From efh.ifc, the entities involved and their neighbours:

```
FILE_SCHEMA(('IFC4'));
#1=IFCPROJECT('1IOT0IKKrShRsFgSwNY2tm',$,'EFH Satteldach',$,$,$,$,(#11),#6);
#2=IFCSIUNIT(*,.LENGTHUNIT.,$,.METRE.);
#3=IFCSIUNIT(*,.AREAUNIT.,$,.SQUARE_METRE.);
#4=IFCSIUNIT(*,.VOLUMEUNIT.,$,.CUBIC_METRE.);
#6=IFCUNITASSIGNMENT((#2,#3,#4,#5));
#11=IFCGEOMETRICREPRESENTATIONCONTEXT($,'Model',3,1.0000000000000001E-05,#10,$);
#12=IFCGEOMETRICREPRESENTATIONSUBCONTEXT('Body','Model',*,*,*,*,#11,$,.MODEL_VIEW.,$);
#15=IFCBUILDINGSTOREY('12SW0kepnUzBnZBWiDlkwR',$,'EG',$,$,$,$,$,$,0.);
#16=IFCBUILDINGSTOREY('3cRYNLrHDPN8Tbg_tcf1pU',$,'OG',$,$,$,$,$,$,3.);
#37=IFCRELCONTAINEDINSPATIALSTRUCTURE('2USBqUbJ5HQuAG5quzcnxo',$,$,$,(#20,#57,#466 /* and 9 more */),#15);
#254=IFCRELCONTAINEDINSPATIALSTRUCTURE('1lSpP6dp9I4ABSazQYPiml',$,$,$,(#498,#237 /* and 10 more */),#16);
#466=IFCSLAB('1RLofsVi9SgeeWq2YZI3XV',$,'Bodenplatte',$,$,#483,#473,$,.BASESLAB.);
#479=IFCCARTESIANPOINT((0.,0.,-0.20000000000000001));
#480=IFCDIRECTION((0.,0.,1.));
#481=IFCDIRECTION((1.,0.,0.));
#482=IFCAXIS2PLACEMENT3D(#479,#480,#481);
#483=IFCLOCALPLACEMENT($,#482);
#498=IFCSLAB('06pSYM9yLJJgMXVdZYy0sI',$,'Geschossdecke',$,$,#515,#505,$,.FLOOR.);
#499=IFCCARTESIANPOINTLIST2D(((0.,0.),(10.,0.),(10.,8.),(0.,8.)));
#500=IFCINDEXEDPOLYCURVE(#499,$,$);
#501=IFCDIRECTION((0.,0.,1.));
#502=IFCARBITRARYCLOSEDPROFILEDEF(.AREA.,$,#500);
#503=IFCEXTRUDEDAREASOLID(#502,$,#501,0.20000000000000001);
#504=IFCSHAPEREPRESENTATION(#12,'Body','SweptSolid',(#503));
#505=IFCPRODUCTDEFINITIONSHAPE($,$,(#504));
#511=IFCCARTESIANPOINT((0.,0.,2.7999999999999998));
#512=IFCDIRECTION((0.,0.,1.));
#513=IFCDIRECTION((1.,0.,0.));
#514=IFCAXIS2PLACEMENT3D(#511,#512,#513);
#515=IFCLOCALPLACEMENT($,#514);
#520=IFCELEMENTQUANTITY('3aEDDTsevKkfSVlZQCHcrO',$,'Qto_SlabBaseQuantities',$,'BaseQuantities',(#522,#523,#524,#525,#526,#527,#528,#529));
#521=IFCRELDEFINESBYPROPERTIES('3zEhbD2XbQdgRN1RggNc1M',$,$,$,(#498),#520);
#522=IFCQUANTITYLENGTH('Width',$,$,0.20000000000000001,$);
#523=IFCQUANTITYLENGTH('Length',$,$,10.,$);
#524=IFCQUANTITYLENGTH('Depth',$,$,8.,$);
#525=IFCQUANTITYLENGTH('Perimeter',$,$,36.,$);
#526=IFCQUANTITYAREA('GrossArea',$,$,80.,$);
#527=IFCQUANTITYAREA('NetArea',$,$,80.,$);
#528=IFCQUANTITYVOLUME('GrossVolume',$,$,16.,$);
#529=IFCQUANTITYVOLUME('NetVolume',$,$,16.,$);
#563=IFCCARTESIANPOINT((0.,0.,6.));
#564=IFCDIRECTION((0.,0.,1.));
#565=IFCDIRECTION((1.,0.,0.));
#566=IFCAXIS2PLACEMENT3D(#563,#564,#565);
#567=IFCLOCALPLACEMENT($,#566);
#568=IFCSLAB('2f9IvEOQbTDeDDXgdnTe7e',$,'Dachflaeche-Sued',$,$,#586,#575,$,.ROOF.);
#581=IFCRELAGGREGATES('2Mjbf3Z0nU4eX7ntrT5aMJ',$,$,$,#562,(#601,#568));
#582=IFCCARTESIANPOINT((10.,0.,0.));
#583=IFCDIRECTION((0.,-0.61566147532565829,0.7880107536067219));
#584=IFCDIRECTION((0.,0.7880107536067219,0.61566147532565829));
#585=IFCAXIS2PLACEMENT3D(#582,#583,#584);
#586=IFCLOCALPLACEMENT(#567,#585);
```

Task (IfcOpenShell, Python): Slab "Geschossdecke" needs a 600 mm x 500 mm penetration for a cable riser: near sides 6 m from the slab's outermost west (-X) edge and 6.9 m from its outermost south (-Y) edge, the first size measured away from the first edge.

```python
import numpy as np
import ifcopenshell
import ifcopenshell.api.feature
import ifcopenshell.api.geometry
import ifcopenshell.api.pset
import ifcopenshell.api.root
import ifcopenshell.geom
import ifcopenshell.util.element
import ifcopenshell.util.placement
import ifcopenshell.util.representation
import ifcopenshell.util.shape
import ifcopenshell.util.unit

model = ifcopenshell.open("efh.ifc")
unit_scale = ifcopenshell.util.unit.calculate_unit_scale(model)
area_scale = ifcopenshell.util.unit.calculate_unit_scale(model, "AREAUNIT")
volume_scale = ifcopenshell.util.unit.calculate_unit_scale(model, "VOLUMEUNIT")
settings = ifcopenshell.geom.settings()


def volume(element):
    """Net volume in cubic metres, openings subtracted."""
    shape = ifcopenshell.geom.create_shape(settings, element)
    return ifcopenshell.util.shape.get_volume(shape.geometry)


slab = model.by_id(498)
before = volume(slab)

# Extent in the slab's own axes, in metres. The edges named are its -X and -Y sides.
slab_shape = ifcopenshell.geom.create_shape(settings, slab)
vertices = ifcopenshell.util.shape.get_vertices(slab_shape.geometry)
x_min, y_min, bottom = vertices.min(axis=0)
top = vertices[:, 2].max()

opening = ifcopenshell.api.root.create_entity(model, ifc_class="IfcOpeningElement", name="Cable riser opening", predefined_type="OPENING")
context = ifcopenshell.util.representation.get_context(model, "Model", "Body", "MODEL_VIEW")
width, depth = 0.6, 0.5
outline = [(0.0, 0.0), (width, 0.0), (width, depth), (0.0, depth), (0.0, 0.0)]
# Overshoot both faces by 50 mm so the cut is clean.
shape = ifcopenshell.api.geometry.add_slab_representation(
    model, context=context, depth=top - bottom + 0.1, polyline=outline
)
ifcopenshell.api.geometry.assign_representation(model, product=opening, representation=shape)

matrix = ifcopenshell.util.placement.get_local_placement(slab.ObjectPlacement)
matrix[:, 3] = matrix @ np.append(np.array([x_min + 6, y_min + 6.9, bottom - 0.05]) / unit_scale, 1.0)
ifcopenshell.api.geometry.edit_object_placement(model, product=opening, matrix=matrix, is_si=False)
ifcopenshell.api.feature.add_feature(model, feature=opening, element=slab)

after = volume(slab)

# Update the slab's stored quantities.
qto = model.by_id(ifcopenshell.util.element.get_pset(slab, "Qto_SlabBaseQuantities", should_inherit=False)["id"])
ifcopenshell.api.pset.edit_qto(model, qto=qto, properties={
    "NetArea": after / (top - bottom) / area_scale,
    "NetVolume": after / volume_scale,
})

print(f"slab volume {before:.3f} -> {after:.3f} m3")

model.write("efh_v2.ifc")
```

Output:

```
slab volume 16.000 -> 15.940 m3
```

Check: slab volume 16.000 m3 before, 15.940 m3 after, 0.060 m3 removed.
